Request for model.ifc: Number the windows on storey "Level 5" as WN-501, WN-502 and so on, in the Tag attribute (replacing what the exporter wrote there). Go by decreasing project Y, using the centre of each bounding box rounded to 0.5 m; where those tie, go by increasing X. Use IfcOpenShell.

First a look at what the model holds.

```python
import ifcopenshell
import ifcopenshell.util.element
import ifcopenshell.util.placement

model = ifcopenshell.open("model.ifc")
print(model.schema)
storey = next(s for s in model.by_type("IfcBuildingStorey") if s.Name == "Level 5")
windows = [e for e in ifcopenshell.util.element.get_decomposition(storey) if e.is_a("IfcWindow")]
for e in sorted(windows, key=lambda e: e.id()):
    origin = ifcopenshell.util.placement.get_local_placement(e.ObjectPlacement)[:3, 3]
    print(e.id(), e.Tag, e.Name, origin.round(2) + 0.0, sep=" | ")
```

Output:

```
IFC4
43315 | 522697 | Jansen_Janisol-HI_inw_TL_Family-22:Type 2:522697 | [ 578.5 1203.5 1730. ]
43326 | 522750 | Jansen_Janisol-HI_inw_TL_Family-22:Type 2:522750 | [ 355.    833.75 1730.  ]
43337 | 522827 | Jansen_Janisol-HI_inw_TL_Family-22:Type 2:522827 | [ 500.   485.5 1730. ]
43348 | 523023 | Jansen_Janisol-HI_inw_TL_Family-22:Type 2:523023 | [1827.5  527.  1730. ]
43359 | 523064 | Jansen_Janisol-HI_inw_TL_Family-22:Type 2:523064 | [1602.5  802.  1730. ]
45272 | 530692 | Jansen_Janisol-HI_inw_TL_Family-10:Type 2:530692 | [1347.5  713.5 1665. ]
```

```python
import ifcopenshell
import ifcopenshell.geom
import ifcopenshell.util.element
import ifcopenshell.util.shape

model = ifcopenshell.open("model.ifc")
settings = ifcopenshell.geom.settings()
settings.set("use-world-coords", True)


def centre(element):
    shape = ifcopenshell.geom.create_shape(settings, element)
    return ifcopenshell.util.shape.get_bbox_centroid(shape.geometry)


storey = next(s for s in model.by_type("IfcBuildingStorey") if s.Name == "Level 5")
windows = [e for e in ifcopenshell.util.element.get_decomposition(storey) if e.is_a("IfcWindow")]

# Insertion points can sit at a corner or the storey origin, so sort by the geometry (in metres).
centres = {e: centre(e) for e in windows}
windows.sort(key=lambda e: (-round(centres[e][1] / 0.5), centres[e][0]))

for i, e in enumerate(windows, start=1):
    number = f"WN-5{i:02d}"
    e.Tag = number
    print(e.id(), number)

model.write("model_edited.ifc")
```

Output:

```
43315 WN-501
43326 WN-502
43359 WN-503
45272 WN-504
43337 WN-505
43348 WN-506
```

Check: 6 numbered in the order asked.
